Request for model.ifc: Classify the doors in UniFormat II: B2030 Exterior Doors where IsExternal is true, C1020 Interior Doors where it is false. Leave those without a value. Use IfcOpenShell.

First a look at what the model holds.

```python
import ifcopenshell
import ifcopenshell.util.element

model = ifcopenshell.open("model.ifc")
print(model.schema)
print("classifications:", [c.Name for c in model.by_type("IfcClassification")])
values = [ifcopenshell.util.element.get_pset(e, "Pset_DoorCommon", "IsExternal") for e in model.by_type("IfcDoor")]
for value in (True, False, None):
    print("IsExternal", value, values.count(value))
```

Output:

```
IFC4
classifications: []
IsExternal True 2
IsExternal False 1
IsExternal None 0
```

```python
import ifcopenshell
import ifcopenshell.api.classification
import ifcopenshell.util.element

model = ifcopenshell.open("model.ifc")

system = ifcopenshell.api.classification.add_classification(model, classification="UniFormat II")

doors = model.by_type("IfcDoor")
external = {e: ifcopenshell.util.element.get_pset(e, "Pset_DoorCommon", "IsExternal") for e in doors}
for flag, code, name in ((True, "B2030", "Exterior Doors"), (False, "C1020", "Interior Doors")):
    products = [e for e in doors if external[e] is flag]
    ifcopenshell.api.classification.add_reference(
        model, products=products, classification=system, identification=code, name=name
    )
    print(code, len(products))

model.write("model_v2.ifc")
```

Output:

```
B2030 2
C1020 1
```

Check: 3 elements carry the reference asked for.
